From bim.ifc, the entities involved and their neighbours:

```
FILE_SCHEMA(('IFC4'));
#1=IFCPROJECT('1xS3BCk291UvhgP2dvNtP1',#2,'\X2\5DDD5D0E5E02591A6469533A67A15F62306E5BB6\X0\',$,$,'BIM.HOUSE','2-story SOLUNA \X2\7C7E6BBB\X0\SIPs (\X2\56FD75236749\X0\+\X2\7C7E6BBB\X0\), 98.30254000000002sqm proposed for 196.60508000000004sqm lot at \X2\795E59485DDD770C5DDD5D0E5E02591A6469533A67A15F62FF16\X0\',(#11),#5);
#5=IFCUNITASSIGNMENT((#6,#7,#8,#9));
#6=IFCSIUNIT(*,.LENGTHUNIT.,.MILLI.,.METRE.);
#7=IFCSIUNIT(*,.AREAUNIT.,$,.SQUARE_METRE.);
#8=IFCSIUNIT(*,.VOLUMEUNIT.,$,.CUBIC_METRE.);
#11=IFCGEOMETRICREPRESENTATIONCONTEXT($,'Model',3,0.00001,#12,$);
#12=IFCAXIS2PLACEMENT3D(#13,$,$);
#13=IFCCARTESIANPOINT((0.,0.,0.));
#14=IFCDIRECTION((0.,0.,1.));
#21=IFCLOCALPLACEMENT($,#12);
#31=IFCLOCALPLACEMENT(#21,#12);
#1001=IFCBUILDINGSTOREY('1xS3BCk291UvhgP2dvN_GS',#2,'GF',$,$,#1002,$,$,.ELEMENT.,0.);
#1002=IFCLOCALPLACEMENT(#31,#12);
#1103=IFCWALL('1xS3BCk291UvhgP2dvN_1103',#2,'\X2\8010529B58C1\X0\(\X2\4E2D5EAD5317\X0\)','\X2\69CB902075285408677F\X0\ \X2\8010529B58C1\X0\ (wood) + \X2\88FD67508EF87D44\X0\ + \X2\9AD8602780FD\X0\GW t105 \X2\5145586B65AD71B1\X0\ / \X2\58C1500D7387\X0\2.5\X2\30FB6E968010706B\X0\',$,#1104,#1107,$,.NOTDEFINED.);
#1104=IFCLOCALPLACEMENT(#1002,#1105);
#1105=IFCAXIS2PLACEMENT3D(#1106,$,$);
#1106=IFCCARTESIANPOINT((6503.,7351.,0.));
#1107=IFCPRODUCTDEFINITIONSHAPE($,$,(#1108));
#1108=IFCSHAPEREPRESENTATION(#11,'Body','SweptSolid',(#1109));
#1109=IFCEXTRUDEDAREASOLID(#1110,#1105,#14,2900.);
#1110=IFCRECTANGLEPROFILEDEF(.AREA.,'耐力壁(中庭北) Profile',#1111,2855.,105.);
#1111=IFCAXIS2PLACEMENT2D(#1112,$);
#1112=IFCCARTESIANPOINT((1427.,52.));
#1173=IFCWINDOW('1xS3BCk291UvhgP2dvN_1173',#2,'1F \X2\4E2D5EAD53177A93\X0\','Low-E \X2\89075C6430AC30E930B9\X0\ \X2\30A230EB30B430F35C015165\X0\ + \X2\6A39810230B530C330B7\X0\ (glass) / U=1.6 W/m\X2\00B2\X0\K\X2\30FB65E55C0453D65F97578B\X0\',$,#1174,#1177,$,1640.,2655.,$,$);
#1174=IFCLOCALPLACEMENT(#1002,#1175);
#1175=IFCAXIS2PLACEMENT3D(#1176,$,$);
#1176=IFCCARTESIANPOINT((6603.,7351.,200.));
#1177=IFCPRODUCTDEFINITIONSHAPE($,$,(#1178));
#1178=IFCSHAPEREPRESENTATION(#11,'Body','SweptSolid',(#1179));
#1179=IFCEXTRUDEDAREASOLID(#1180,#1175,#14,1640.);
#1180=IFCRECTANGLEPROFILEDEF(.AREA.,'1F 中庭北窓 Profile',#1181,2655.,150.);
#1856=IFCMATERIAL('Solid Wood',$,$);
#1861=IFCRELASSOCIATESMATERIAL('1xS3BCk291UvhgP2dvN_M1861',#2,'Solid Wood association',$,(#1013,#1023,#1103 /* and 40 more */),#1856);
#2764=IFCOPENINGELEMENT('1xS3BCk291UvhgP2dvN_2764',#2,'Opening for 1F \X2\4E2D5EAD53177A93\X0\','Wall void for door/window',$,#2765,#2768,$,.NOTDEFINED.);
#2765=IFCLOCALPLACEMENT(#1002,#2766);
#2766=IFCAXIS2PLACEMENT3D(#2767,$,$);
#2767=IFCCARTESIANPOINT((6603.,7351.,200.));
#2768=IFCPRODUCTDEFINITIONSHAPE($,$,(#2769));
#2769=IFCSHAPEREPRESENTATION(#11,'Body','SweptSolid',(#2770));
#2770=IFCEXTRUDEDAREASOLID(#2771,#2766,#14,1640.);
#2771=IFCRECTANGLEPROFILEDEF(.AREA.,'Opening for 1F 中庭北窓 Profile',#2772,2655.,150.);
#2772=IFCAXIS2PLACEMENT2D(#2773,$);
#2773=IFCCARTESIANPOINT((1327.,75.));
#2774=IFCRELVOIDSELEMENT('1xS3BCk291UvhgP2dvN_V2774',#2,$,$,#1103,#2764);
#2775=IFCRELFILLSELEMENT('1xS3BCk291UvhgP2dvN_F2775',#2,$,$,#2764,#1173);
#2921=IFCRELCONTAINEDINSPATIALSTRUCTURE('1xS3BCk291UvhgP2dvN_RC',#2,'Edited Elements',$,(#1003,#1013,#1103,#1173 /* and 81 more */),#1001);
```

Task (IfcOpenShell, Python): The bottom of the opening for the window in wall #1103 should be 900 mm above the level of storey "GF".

```python
import numpy as np
import ifcopenshell
import ifcopenshell.api.geometry
import ifcopenshell.geom
import ifcopenshell.util.element
import ifcopenshell.util.placement
import ifcopenshell.util.shape
import ifcopenshell.util.unit

model = ifcopenshell.open("bim.ifc")
unit_scale = ifcopenshell.util.unit.calculate_unit_scale(model)

window = model.by_guid("1xS3BCk291UvhgP2dvN_1173")
opening = window.FillsVoids[0].RelatingOpeningElement
storey = ifcopenshell.util.element.get_container(window, ifc_class="IfcBuildingStorey")
level = ifcopenshell.util.placement.get_local_placement(storey.ObjectPlacement)[2, 3]

# The opening's origin need not be at the sill, so measure its lowest point.
shape = ifcopenshell.geom.create_shape(ifcopenshell.geom.settings(), opening)
bottom = ifcopenshell.util.shape.get_shape_bottom_elevation(shape, shape.geometry) / unit_scale
dz = level + 0.9 / unit_scale - bottom

shift = np.array([0.0, 0.0, dz])
# The window is not placed relative to its opening, so move both.
for product in (opening, window):
    matrix = ifcopenshell.util.placement.get_local_placement(product.ObjectPlacement)
    matrix[:3, 3] += shift
    ifcopenshell.api.geometry.edit_object_placement(model, product=product, matrix=matrix, is_si=False)

print(f"moved by {dz * unit_scale:+.3f} m")

model.write("bim_v2.ifc")
```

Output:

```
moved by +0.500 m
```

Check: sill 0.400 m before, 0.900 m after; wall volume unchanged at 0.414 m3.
